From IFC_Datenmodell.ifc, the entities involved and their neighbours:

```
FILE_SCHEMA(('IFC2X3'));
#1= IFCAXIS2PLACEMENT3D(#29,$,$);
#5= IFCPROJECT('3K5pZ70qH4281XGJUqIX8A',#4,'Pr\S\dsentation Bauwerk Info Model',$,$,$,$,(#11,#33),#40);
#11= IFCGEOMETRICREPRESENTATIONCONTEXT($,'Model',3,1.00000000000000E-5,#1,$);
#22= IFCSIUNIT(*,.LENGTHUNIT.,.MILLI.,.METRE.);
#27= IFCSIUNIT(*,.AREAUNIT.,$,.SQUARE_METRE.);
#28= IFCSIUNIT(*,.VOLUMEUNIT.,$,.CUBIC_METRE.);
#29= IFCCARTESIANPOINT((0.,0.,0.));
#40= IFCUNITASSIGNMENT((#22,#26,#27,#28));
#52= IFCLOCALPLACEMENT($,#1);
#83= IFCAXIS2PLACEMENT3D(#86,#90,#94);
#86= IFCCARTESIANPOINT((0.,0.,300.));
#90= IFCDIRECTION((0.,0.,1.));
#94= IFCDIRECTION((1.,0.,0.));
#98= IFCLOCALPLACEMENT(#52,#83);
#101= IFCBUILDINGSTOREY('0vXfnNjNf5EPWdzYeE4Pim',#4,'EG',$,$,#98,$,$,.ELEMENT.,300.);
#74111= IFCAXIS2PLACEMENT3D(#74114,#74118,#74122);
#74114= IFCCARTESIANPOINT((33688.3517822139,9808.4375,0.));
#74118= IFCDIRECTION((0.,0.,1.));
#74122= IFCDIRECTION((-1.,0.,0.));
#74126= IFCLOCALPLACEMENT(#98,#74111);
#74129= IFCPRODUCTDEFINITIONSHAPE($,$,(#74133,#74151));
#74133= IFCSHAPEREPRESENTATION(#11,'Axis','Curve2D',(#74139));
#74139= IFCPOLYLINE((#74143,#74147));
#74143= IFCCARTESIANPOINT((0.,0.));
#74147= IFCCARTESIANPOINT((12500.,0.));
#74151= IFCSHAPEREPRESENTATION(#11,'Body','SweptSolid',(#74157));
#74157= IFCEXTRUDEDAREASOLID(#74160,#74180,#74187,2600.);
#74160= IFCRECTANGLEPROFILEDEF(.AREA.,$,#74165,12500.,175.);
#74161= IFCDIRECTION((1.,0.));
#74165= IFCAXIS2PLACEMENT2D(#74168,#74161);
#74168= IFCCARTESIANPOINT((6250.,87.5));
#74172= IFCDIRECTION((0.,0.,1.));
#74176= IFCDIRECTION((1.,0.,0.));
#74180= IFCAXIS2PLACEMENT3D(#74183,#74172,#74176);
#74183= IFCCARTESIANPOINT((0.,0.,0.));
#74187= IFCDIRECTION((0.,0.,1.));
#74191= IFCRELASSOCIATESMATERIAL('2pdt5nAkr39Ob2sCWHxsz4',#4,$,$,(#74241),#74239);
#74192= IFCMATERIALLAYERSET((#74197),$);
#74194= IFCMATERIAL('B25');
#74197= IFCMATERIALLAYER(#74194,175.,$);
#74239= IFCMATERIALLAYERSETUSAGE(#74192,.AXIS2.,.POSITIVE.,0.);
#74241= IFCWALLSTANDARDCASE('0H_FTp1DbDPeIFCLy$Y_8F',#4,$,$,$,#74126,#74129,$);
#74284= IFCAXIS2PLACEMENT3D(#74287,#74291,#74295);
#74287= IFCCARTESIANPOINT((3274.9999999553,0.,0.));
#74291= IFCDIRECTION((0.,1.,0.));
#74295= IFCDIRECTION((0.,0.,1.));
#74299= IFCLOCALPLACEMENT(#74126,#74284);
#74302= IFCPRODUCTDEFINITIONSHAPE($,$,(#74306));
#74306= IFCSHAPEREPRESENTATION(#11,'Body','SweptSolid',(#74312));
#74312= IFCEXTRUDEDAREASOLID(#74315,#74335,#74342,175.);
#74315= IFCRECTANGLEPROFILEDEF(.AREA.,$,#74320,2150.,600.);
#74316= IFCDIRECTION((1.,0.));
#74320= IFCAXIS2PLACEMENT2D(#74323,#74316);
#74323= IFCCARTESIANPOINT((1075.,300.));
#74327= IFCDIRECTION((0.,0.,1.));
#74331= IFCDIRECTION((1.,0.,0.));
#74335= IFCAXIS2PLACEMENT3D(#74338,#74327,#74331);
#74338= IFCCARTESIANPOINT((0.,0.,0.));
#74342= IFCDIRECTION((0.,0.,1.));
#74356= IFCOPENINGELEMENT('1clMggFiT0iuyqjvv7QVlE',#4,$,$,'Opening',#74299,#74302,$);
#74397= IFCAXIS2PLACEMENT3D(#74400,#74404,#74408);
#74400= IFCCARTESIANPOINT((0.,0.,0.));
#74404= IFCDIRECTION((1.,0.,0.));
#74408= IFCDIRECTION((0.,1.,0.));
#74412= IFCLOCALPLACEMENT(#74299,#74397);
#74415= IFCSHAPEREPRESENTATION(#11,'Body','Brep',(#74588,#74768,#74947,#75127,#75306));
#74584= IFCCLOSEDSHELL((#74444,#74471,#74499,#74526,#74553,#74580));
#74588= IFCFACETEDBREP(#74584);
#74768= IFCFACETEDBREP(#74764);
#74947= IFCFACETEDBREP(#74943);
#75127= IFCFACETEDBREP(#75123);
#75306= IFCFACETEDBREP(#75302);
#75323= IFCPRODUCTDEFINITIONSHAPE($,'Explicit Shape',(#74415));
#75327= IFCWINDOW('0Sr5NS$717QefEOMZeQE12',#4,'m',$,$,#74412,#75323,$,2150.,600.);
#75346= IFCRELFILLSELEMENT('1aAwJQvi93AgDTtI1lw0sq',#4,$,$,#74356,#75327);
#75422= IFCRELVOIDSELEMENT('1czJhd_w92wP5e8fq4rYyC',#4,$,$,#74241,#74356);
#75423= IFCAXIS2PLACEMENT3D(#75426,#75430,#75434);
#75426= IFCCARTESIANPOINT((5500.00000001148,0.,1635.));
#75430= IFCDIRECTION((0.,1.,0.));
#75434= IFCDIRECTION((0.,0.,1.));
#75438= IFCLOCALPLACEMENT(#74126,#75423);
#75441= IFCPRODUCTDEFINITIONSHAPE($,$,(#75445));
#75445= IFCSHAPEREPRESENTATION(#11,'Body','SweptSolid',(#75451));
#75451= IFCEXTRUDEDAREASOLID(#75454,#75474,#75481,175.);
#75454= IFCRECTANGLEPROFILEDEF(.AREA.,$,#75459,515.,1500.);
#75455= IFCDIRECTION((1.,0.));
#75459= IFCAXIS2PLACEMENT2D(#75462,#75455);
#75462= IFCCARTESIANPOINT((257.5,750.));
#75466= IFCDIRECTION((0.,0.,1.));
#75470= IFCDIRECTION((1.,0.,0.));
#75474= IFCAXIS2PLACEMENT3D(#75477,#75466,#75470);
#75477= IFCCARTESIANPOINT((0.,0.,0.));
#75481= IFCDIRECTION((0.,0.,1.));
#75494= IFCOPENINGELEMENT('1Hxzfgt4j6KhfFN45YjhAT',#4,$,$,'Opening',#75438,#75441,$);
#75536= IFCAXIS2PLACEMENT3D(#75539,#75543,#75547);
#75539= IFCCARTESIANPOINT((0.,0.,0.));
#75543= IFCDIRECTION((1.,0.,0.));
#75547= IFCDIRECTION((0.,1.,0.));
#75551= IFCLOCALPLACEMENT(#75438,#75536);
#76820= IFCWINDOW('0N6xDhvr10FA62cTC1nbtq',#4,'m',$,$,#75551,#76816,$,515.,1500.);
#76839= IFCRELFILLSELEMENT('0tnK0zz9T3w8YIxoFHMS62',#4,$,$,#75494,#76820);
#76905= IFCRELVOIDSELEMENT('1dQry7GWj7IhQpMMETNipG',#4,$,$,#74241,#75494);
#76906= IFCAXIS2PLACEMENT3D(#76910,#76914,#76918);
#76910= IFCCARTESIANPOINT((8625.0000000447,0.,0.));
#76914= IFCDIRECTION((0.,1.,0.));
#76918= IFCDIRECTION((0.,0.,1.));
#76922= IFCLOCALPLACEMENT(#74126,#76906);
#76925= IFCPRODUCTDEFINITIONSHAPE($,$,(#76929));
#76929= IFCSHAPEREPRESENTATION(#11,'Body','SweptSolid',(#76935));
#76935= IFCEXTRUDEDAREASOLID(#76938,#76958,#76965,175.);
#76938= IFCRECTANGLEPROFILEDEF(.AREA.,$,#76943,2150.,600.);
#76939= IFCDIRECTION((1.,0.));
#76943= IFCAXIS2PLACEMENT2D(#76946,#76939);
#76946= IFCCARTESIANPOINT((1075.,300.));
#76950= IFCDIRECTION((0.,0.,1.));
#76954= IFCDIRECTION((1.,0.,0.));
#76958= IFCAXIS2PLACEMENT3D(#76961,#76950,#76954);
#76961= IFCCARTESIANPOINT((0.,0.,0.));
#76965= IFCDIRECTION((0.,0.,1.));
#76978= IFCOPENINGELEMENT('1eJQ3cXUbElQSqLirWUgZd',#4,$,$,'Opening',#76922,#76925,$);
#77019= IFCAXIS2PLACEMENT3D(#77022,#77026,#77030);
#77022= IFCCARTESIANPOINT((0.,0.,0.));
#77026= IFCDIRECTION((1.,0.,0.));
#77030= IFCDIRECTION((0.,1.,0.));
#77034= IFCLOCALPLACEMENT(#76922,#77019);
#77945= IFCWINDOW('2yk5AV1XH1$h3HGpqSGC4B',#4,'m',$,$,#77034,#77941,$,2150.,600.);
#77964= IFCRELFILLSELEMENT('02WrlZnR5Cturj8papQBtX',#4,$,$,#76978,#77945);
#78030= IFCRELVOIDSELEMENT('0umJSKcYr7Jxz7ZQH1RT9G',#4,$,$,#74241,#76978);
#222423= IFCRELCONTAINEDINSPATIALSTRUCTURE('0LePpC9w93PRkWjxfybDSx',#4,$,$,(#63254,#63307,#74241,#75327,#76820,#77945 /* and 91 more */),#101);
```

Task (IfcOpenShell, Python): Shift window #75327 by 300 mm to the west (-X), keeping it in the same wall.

```python
import ifcopenshell
import ifcopenshell.api.geometry
import ifcopenshell.util.placement

model = ifcopenshell.open("IFC_Datenmodell.ifc")

window = model.by_guid("0Sr5NS$717QefEOMZeQE12")
opening = window.FillsVoids[0].RelatingOpeningElement
wall = opening.VoidsElements[0].RelatingBuildingElement

wall_matrix = ifcopenshell.util.placement.get_local_placement(wall.ObjectPlacement)
shift = wall_matrix[:3, 0] * 300.0
before = ifcopenshell.util.placement.get_local_placement(window.ObjectPlacement)[:3, 3].copy()

# The window is placed relative to its opening, so it follows when the opening moves.
matrix = ifcopenshell.util.placement.get_local_placement(opening.ObjectPlacement)
matrix[:3, 3] += shift
ifcopenshell.api.geometry.edit_object_placement(
    model, product=opening, matrix=matrix, is_si=False, should_transform_children=True
)

after = ifcopenshell.util.placement.get_local_placement(window.ObjectPlacement)[:3, 3]
print("window moved by", (after - before).round(3) + 0.0)

model.write("IFC_Datenmodell-out.ifc")
```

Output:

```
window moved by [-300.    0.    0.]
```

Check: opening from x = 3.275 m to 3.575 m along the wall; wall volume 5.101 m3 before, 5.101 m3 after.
